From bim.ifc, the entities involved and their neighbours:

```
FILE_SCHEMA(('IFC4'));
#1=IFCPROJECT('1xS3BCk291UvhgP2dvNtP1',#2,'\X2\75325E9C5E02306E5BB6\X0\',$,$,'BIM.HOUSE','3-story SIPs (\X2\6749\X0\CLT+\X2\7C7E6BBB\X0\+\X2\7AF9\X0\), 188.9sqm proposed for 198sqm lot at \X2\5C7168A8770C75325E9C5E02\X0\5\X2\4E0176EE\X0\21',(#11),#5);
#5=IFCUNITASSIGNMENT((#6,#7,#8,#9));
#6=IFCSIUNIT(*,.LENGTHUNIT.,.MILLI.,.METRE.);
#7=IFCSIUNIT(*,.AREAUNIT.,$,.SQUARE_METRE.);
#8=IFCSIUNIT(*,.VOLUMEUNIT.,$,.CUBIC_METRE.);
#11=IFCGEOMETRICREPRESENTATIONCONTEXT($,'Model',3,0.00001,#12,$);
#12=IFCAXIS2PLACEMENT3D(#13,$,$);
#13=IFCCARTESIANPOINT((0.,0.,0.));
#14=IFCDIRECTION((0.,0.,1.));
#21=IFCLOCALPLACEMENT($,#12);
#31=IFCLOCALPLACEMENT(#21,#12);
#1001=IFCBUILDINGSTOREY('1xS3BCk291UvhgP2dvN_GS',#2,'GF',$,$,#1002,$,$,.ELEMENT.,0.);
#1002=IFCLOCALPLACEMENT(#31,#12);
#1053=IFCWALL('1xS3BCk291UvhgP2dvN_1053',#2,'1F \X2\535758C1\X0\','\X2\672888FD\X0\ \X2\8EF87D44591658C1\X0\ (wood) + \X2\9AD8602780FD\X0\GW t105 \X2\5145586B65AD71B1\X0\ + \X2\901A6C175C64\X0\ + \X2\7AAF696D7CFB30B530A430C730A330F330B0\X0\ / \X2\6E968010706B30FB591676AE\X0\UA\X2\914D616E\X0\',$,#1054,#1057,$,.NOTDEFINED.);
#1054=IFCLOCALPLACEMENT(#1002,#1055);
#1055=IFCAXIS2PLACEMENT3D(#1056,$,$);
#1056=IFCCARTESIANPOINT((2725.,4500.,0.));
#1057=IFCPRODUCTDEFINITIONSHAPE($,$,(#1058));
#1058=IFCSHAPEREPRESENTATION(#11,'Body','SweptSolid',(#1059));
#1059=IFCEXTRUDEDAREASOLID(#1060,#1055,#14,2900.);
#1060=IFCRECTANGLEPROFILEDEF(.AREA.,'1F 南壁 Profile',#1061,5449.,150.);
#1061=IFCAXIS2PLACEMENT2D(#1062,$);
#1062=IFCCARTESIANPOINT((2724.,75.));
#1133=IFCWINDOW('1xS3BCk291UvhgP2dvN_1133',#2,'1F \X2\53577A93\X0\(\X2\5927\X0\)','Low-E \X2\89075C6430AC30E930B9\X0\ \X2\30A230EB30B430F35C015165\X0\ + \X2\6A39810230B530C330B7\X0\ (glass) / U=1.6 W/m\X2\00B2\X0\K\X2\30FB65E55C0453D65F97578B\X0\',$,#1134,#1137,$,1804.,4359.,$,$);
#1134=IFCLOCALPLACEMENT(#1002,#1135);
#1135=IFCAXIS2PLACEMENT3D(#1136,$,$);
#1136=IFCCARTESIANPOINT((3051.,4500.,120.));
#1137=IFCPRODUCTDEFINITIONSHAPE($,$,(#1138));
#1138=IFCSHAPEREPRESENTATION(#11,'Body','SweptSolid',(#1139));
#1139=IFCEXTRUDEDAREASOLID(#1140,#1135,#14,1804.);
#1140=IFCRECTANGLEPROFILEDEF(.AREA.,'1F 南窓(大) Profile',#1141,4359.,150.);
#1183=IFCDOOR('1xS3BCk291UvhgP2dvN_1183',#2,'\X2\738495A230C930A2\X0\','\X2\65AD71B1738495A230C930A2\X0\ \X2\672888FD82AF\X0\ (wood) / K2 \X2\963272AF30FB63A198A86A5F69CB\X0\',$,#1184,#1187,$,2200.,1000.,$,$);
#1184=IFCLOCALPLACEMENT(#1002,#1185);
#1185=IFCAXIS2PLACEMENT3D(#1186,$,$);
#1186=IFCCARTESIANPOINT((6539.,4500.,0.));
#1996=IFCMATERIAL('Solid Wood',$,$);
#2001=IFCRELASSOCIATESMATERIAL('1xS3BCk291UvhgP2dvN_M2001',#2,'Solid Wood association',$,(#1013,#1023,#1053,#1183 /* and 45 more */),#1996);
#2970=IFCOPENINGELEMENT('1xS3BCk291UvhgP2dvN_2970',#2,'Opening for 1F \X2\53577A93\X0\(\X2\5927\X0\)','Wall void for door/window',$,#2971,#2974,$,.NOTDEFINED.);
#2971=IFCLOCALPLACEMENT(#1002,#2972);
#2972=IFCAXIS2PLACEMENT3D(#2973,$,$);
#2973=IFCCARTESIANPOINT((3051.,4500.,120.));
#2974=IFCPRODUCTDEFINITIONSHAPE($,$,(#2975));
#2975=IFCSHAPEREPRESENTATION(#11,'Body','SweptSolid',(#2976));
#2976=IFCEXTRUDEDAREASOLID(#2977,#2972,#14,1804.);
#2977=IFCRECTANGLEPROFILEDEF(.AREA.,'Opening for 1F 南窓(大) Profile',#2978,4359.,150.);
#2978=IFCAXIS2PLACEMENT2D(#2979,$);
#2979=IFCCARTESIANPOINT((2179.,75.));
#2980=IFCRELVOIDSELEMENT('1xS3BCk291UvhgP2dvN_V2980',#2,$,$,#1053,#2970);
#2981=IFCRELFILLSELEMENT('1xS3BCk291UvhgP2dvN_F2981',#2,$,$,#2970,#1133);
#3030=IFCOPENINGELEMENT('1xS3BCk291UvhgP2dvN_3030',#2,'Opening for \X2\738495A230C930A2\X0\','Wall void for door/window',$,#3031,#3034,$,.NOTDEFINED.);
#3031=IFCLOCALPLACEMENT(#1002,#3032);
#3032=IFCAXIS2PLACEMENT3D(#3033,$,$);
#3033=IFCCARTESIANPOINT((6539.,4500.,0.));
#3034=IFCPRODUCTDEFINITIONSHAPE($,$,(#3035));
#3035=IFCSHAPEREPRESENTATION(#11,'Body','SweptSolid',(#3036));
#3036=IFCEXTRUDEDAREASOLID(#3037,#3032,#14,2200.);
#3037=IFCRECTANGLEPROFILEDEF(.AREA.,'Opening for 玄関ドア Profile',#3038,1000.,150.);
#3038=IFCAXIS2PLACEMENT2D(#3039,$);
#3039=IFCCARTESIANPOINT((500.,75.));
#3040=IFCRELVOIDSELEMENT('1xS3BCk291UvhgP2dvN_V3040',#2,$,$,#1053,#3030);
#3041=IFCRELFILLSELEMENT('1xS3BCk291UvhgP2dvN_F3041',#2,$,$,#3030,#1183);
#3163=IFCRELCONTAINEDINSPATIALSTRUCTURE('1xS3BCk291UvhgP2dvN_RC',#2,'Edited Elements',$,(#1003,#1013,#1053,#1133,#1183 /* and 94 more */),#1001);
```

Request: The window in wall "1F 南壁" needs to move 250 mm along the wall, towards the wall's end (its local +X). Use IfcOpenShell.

```python
import ifcopenshell
import ifcopenshell.api.geometry
import ifcopenshell.util.placement
import ifcopenshell.util.unit

model = ifcopenshell.open("bim.ifc")
unit_scale = ifcopenshell.util.unit.calculate_unit_scale(model)

window = model.by_guid("1xS3BCk291UvhgP2dvN_1133")
opening = window.FillsVoids[0].RelatingOpeningElement
wall = opening.VoidsElements[0].RelatingBuildingElement

wall_matrix = ifcopenshell.util.placement.get_local_placement(wall.ObjectPlacement)
shift = wall_matrix[:3, 0] * 0.25 / unit_scale
before = ifcopenshell.util.placement.get_local_placement(window.ObjectPlacement)[:3, 3].copy()

# The window is not placed relative to its opening, so move both.
for product in (opening, window):
    matrix = ifcopenshell.util.placement.get_local_placement(product.ObjectPlacement)
    matrix[:3, 3] += shift
    ifcopenshell.api.geometry.edit_object_placement(model, product=product, matrix=matrix, is_si=False)

after = ifcopenshell.util.placement.get_local_placement(window.ObjectPlacement)[:3, 3]
print("window moved by", (after - before).round(3) + 0.0)

model.write("bim_edited.ifc")
```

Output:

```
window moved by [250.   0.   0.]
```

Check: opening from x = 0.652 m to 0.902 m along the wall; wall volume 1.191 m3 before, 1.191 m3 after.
